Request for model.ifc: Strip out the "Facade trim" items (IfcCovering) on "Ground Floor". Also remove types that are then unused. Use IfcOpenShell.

First a look at what the model holds.

```python
import ifcopenshell
import ifcopenshell.util.element

model = ifcopenshell.open("model.ifc")
print(model.schema)
storey = next(s for s in model.by_type("IfcBuildingStorey") if s.Name == "Ground Floor")
coverings = [e for e in ifcopenshell.util.element.get_decomposition(storey) if e.is_a("IfcCovering")]
seen = {}
for e in coverings:
    element_type = ifcopenshell.util.element.get_type(e)
    name = element_type.Name if element_type not in (None, e) else None
    seen[name] = seen.get(name, 0) + 1
for name, count in sorted(seen.items(), key=str):
    print(count, "x", name)
```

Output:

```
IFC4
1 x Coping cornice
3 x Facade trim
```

```python
import ifcopenshell
import ifcopenshell.api.root
import ifcopenshell.util.element

model = ifcopenshell.open("model.ifc")

storey = next(s for s in model.by_type("IfcBuildingStorey") if s.Name == "Ground Floor")
coverings = [e for e in ifcopenshell.util.element.get_decomposition(storey) if e.is_a("IfcCovering")]
targets = [e for e in coverings if (t := ifcopenshell.util.element.get_type(e)) not in (None, e) and t.Name == "Facade trim"]
types = {ifcopenshell.util.element.get_type(e) for e in targets} - {None, *targets}

for e in targets:
    ifcopenshell.api.root.remove_product(model, product=e)
print(len(targets), "removed")

unused = [t for t in types if not ifcopenshell.util.element.get_types(t)]
for t in unused:
    ifcopenshell.api.root.remove_product(model, product=t)
print(len(unused), "unused types removed")

model.write("model_v2.ifc")
```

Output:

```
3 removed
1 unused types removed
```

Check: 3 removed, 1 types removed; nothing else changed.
